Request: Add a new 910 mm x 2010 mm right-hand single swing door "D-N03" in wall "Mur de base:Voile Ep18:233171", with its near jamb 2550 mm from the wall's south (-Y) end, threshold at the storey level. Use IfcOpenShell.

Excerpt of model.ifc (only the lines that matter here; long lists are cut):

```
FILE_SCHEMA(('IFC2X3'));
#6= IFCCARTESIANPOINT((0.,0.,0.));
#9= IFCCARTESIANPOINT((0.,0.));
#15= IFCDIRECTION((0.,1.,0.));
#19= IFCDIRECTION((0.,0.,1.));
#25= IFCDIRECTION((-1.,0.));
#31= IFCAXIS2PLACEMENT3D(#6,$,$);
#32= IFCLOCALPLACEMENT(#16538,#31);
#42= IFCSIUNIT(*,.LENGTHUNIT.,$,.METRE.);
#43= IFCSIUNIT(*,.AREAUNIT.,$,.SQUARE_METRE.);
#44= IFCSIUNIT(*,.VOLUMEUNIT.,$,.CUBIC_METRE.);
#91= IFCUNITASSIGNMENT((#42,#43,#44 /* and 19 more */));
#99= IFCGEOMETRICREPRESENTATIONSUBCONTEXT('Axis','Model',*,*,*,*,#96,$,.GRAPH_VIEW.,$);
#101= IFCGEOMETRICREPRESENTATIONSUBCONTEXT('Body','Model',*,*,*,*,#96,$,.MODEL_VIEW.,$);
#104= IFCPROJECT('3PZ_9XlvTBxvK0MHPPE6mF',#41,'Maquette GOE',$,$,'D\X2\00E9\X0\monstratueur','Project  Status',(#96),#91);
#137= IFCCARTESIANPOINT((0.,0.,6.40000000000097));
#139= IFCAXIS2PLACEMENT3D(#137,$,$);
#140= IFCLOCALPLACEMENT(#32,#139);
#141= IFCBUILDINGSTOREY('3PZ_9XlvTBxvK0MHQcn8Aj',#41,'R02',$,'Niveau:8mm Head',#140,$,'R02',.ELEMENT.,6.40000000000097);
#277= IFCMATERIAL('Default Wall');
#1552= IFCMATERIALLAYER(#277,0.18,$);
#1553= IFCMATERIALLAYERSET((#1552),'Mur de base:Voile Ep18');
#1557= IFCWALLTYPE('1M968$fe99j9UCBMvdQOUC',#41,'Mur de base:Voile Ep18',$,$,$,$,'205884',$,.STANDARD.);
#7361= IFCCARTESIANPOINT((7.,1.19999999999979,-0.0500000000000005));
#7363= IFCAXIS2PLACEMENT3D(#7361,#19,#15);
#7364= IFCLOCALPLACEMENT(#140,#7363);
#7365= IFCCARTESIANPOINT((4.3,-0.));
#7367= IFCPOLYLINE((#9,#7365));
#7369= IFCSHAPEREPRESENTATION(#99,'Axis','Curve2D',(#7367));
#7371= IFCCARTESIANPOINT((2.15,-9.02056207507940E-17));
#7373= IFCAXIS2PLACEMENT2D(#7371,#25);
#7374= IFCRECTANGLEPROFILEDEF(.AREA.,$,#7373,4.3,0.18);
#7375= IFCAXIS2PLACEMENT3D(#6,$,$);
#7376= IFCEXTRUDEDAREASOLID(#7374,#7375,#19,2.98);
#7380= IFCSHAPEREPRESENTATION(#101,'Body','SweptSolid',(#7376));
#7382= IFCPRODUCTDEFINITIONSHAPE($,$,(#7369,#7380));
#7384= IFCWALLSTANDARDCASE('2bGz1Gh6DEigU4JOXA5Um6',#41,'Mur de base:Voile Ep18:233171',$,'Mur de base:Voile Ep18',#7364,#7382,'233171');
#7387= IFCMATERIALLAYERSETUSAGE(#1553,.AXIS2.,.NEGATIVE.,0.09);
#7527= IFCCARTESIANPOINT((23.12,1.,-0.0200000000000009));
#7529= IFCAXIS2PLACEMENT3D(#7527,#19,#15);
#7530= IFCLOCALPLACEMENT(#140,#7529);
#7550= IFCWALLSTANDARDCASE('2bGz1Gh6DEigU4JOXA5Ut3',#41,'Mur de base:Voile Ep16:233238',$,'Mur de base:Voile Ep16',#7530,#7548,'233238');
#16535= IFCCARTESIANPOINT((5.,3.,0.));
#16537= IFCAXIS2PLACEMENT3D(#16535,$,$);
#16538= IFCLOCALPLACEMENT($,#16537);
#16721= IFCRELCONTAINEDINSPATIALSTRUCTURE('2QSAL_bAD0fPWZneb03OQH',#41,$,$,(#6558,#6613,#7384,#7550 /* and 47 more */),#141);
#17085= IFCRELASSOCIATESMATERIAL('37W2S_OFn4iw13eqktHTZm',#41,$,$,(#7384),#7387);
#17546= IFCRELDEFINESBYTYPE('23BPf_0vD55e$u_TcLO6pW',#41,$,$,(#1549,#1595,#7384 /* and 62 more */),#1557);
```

```python
import numpy as np
import ifcopenshell
import ifcopenshell.api.feature
import ifcopenshell.api.geometry
import ifcopenshell.api.root
import ifcopenshell.api.spatial
import ifcopenshell.api.type
import ifcopenshell.geom
import ifcopenshell.util.element
import ifcopenshell.util.placement
import ifcopenshell.util.representation
import ifcopenshell.util.shape
import ifcopenshell.util.unit

model = ifcopenshell.open("model.ifc")
unit_scale = ifcopenshell.util.unit.calculate_unit_scale(model)
settings = ifcopenshell.geom.settings()


def volume(element):
    """Net volume in cubic metres, openings subtracted."""
    shape = ifcopenshell.geom.create_shape(settings, element)
    return ifcopenshell.util.shape.get_volume(shape.geometry)


wall = model.by_guid("2bGz1Gh6DEigU4JOXA5Um6")
storey = ifcopenshell.util.element.get_container(wall, ifc_class="IfcBuildingStorey")
context = ifcopenshell.util.representation.get_context(model, "Model", "Body", "MODEL_VIEW")
before = volume(wall)

width, height, from_end, sill = 0.91, 2.01, 2.55, 0.0  # metres

# The wall runs along its own X axis, and the end named is its -X end.
wall_shape = ifcopenshell.geom.create_shape(settings, wall)
x, y, z = ifcopenshell.util.shape.get_vertices(wall_shape.geometry).T
start = x.min() + from_end
face, thickness = float(y.min()), float(y.max() - y.min())
wall_matrix = ifcopenshell.util.placement.get_local_placement(wall.ObjectPlacement)
level = ifcopenshell.util.placement.get_local_placement(storey.ObjectPlacement)[2, 3]


def in_wall(x, y):
    """Placement at x, y metres in the wall's axes, at sill height."""
    matrix = wall_matrix.copy()
    matrix[:, 3] = wall_matrix @ np.array([x / unit_scale, y / unit_scale, 0.0, 1.0])
    matrix[2, 3] = level + sill / unit_scale
    return matrix


# Opening: a box that overshoots both wall faces by 50 mm.
opening = ifcopenshell.api.root.create_entity(model, ifc_class="IfcOpeningElement")
box = ifcopenshell.api.geometry.add_wall_representation(
    model, context=context, length=width, height=height, thickness=thickness + 0.1
)
ifcopenshell.api.geometry.assign_representation(model, product=opening, representation=box)
ifcopenshell.api.geometry.edit_object_placement(model, product=opening, matrix=in_wall(start, face - 0.05), is_si=False)
ifcopenshell.api.feature.add_feature(model, feature=opening, element=wall)

door = ifcopenshell.api.root.create_entity(model, ifc_class="IfcDoor", name="D-N03")
door.OverallWidth, door.OverallHeight = width / unit_scale, height / unit_scale
body = ifcopenshell.api.geometry.add_door_representation(
    model,
    context=context,
    overall_width=door.OverallWidth,
    overall_height=door.OverallHeight,
    operation_type="SINGLE_SWING_RIGHT",
    lining_properties={"LiningDepth": thickness / unit_scale, "ThresholdDepth": thickness / unit_scale},
)
ifcopenshell.api.geometry.assign_representation(model, product=door, representation=body)
ifcopenshell.api.spatial.assign_container(model, products=[door], relating_structure=storey)
fills = ifcopenshell.api.feature.add_filling(model, opening=opening, element=door)
fills.OwnerHistory = door.OwnerHistory  # required in IFC2X3

# IFC2X3 keeps the operation on the door style.
style = ifcopenshell.api.root.create_entity(model, ifc_class="IfcDoorStyle", name="D-N03")
style.OperationType, style.ConstructionType = "SINGLE_SWING_RIGHT", "NOTDEFINED"
style.ParameterTakesPrecedence = style.Sizeable = False
ifcopenshell.api.type.assign_type(model, related_objects=[door], relating_type=style)

# The lining spans the wall, so the door starts at the wall face.
ifcopenshell.api.geometry.edit_object_placement(model, product=door, matrix=in_wall(start, face), is_si=False)

after = volume(wall)

print(f"wall volume {before:.3f} -> {after:.3f} m3")

model.write("model_v2.ifc")
```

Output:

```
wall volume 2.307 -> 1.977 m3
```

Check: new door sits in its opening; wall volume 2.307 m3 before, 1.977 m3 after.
